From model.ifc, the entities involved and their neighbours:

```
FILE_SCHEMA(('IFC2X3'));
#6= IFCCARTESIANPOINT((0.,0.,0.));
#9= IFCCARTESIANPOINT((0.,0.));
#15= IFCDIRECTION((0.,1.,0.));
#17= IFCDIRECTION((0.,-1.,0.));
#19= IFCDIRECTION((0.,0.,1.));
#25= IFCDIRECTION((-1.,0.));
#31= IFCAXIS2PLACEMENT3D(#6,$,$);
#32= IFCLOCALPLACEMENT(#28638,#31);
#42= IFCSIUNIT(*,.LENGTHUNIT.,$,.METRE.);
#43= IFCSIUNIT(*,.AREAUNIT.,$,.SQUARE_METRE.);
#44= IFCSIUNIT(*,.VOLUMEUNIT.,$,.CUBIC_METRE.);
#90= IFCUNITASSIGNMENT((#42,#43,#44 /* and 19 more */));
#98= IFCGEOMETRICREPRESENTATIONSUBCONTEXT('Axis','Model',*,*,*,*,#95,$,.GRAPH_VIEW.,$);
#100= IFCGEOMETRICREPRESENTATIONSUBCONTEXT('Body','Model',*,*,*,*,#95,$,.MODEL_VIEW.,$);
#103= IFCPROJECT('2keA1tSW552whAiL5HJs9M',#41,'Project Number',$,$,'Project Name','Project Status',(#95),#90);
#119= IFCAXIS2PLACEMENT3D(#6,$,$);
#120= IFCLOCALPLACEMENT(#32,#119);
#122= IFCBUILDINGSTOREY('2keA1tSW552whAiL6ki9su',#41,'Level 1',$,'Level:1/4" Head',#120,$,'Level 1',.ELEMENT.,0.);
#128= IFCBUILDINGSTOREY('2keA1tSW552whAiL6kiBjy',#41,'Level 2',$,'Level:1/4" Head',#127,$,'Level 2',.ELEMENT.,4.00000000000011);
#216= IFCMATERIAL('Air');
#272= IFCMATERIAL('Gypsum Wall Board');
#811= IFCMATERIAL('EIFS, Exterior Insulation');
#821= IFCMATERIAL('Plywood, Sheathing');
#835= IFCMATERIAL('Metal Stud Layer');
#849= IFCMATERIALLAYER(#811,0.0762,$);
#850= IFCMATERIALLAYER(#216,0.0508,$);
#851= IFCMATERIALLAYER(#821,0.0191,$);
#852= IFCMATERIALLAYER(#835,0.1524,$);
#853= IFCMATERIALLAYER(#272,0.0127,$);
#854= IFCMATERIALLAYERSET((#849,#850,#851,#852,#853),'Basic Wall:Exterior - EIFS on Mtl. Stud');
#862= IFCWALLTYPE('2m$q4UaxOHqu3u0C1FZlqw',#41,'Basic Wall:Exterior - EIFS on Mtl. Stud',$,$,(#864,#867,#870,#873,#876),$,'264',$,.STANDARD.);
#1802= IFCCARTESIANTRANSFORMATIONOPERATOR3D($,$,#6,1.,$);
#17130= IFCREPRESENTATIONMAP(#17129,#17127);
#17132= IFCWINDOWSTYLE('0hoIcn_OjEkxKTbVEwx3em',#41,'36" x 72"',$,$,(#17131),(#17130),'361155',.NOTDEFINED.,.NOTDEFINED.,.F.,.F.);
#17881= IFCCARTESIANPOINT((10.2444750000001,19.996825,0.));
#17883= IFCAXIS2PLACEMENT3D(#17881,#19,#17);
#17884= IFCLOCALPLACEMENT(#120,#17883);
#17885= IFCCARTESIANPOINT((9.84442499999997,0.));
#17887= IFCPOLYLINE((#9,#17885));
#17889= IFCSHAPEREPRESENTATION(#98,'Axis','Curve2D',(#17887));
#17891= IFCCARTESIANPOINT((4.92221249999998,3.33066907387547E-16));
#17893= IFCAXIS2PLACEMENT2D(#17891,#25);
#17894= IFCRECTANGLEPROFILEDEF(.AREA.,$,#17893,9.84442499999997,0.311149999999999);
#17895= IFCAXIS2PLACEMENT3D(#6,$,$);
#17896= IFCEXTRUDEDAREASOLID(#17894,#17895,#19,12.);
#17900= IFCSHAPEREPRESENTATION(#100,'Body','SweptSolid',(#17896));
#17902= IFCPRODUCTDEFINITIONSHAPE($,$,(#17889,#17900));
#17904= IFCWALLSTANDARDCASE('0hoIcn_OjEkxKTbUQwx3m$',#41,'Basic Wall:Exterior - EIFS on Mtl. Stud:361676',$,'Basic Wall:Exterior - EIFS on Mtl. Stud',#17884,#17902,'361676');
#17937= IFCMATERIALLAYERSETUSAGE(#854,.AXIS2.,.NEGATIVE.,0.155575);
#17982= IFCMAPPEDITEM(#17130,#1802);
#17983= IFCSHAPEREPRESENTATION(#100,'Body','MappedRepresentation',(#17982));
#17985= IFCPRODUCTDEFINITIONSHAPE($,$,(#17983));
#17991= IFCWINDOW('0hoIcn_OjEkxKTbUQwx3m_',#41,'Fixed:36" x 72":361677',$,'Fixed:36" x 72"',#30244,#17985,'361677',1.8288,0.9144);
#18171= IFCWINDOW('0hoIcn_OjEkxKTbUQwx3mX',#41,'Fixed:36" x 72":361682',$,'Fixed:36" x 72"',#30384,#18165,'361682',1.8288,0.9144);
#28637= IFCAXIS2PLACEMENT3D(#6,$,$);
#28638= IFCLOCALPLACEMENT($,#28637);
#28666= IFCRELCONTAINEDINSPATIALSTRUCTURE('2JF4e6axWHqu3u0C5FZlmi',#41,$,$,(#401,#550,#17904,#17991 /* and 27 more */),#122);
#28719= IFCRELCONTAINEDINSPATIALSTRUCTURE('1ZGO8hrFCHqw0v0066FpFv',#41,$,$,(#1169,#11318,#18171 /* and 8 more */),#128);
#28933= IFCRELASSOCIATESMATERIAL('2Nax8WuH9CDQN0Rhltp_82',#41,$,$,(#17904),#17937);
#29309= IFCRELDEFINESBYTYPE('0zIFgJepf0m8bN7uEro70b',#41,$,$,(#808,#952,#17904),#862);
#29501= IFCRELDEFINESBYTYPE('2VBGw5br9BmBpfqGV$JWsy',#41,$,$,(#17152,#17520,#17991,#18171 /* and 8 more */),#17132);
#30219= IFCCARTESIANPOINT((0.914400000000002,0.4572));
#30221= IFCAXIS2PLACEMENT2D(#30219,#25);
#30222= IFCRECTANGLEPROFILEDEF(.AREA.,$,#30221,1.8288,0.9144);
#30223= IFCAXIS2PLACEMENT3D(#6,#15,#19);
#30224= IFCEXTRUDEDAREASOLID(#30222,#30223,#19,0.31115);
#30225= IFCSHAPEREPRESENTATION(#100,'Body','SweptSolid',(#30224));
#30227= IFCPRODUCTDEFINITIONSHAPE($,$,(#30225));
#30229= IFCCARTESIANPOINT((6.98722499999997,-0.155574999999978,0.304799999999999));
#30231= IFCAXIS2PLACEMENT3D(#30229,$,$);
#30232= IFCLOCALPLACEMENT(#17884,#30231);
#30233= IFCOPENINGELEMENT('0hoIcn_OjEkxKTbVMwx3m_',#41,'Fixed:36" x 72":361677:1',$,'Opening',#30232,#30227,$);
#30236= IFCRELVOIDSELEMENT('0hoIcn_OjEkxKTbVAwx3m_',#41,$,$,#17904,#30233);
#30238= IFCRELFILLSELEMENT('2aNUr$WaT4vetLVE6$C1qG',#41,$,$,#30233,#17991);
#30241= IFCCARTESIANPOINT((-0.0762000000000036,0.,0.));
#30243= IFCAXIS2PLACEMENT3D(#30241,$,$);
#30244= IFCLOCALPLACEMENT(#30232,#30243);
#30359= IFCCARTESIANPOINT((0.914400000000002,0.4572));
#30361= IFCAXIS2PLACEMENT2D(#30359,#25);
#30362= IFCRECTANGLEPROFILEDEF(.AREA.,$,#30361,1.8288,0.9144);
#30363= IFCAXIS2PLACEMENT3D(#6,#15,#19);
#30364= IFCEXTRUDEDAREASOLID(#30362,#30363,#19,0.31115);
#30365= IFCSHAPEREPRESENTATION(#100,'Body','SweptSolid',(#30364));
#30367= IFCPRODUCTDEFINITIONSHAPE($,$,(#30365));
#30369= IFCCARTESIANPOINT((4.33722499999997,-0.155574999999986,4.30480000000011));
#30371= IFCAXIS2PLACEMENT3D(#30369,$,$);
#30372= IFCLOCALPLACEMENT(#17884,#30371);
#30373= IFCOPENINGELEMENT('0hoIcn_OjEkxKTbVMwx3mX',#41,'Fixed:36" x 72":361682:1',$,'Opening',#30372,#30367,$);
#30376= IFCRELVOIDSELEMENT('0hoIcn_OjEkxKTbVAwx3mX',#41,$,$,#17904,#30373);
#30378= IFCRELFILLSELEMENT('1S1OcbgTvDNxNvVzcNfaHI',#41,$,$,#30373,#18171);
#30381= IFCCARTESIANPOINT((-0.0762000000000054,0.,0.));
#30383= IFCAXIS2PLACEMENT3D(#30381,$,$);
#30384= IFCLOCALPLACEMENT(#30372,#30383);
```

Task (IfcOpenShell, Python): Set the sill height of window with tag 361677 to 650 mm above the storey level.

```python
import numpy as np
import ifcopenshell
import ifcopenshell.api.geometry
import ifcopenshell.geom
import ifcopenshell.util.element
import ifcopenshell.util.placement
import ifcopenshell.util.shape
import ifcopenshell.util.unit

model = ifcopenshell.open("model.ifc")
unit_scale = ifcopenshell.util.unit.calculate_unit_scale(model)

window = model.by_guid("0hoIcn_OjEkxKTbUQwx3m_")
opening = window.FillsVoids[0].RelatingOpeningElement
storey = ifcopenshell.util.element.get_container(window, ifc_class="IfcBuildingStorey")
level = ifcopenshell.util.placement.get_local_placement(storey.ObjectPlacement)[2, 3]

# The opening's origin need not be at the sill, so measure its lowest point.
shape = ifcopenshell.geom.create_shape(ifcopenshell.geom.settings(), opening)
bottom = ifcopenshell.util.shape.get_shape_bottom_elevation(shape, shape.geometry) / unit_scale
dz = level + 0.65 / unit_scale - bottom

shift = np.array([0.0, 0.0, dz])
# The window is placed relative to its opening, so it follows when the opening moves.
matrix = ifcopenshell.util.placement.get_local_placement(opening.ObjectPlacement)
matrix[:3, 3] += shift
ifcopenshell.api.geometry.edit_object_placement(
    model, product=opening, matrix=matrix, is_si=False, should_transform_children=True
)

print(f"moved by {dz * unit_scale:+.3f} m")

model.write("model_updated.ifc")
```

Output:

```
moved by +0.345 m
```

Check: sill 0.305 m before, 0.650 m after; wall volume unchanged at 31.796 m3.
